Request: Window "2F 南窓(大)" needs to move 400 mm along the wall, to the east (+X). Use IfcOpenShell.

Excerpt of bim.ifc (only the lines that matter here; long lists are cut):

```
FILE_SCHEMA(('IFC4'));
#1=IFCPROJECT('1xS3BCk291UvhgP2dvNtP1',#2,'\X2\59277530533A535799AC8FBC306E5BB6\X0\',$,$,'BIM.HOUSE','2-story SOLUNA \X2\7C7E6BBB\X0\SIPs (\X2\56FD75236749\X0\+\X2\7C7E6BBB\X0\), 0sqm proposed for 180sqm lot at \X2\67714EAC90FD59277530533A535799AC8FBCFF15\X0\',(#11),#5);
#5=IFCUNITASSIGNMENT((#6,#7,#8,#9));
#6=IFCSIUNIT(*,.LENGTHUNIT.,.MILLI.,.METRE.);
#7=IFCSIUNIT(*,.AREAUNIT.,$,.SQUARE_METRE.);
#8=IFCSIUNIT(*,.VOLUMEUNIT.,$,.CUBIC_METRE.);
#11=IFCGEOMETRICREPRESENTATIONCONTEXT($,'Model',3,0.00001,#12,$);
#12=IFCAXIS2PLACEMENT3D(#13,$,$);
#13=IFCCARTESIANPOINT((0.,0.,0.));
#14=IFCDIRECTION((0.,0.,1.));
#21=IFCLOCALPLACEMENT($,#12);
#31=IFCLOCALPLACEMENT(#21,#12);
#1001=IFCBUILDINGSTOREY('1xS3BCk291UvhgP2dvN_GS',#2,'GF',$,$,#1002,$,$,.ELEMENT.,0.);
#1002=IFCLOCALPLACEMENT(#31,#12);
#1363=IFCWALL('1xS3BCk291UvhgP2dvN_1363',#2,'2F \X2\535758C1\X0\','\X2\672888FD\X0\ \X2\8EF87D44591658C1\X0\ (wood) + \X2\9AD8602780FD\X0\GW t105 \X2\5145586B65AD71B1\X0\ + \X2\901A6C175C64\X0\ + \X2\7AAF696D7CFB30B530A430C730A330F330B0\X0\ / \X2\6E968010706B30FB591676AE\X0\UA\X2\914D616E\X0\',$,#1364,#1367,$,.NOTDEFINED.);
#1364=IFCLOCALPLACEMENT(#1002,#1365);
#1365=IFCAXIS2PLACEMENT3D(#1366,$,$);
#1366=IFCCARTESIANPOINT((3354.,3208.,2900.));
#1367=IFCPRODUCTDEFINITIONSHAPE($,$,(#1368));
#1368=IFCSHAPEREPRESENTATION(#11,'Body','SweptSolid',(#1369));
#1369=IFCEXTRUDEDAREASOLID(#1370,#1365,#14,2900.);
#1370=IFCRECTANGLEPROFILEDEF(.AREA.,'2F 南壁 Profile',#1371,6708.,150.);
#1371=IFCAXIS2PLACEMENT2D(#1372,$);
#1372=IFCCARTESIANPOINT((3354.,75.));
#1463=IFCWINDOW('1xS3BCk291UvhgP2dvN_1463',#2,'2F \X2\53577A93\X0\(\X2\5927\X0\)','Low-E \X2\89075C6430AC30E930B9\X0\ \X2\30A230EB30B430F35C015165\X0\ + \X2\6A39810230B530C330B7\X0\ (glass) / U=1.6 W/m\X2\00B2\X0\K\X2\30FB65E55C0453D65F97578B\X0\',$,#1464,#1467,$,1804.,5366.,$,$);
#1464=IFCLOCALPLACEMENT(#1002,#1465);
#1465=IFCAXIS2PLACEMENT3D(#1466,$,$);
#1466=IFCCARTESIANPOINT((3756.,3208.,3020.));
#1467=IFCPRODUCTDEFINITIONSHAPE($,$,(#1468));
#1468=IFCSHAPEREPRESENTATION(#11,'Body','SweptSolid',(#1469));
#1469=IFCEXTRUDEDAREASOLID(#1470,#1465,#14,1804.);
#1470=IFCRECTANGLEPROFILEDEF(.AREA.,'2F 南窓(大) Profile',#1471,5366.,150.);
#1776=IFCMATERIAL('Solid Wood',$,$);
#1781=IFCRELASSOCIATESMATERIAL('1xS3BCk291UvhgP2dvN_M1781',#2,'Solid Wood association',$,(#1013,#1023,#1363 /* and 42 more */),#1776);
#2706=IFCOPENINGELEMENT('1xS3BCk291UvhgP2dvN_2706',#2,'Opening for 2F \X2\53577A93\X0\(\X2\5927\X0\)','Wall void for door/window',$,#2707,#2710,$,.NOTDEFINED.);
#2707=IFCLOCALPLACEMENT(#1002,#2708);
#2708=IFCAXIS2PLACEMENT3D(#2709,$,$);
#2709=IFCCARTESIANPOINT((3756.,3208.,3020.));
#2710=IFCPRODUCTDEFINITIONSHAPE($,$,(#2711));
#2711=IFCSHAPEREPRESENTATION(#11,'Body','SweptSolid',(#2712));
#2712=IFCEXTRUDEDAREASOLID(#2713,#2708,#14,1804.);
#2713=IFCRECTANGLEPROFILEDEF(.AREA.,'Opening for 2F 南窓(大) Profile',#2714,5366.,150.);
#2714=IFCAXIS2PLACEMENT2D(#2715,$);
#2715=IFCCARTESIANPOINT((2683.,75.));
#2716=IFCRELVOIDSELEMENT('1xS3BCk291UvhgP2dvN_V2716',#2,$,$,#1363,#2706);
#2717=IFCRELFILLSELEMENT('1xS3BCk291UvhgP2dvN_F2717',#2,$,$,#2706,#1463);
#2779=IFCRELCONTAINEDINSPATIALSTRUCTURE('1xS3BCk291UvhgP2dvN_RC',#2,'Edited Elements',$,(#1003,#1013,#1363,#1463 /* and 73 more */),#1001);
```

```python
import ifcopenshell
import ifcopenshell.api.geometry
import ifcopenshell.util.placement

model = ifcopenshell.open("bim.ifc")

window = model.by_id(1463)
opening = window.FillsVoids[0].RelatingOpeningElement
wall = opening.VoidsElements[0].RelatingBuildingElement

wall_matrix = ifcopenshell.util.placement.get_local_placement(wall.ObjectPlacement)
shift = wall_matrix[:3, 0] * 400.0
before = ifcopenshell.util.placement.get_local_placement(window.ObjectPlacement)[:3, 3].copy()

# The window is not placed relative to its opening, so move both.
for product in (opening, window):
    matrix = ifcopenshell.util.placement.get_local_placement(product.ObjectPlacement)
    matrix[:3, 3] += shift
    ifcopenshell.api.geometry.edit_object_placement(model, product=product, matrix=matrix, is_si=False)

after = ifcopenshell.util.placement.get_local_placement(window.ObjectPlacement)[:3, 3]
print("window moved by", (after - before).round(3) + 0.0)

model.write("bim_edited.ifc")
```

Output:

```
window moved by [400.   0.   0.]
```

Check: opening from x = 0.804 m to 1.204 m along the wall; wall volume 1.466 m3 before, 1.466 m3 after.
